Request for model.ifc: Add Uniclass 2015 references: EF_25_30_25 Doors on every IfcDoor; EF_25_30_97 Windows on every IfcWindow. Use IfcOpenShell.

First a look at what the model holds.

```python
import ifcopenshell

model = ifcopenshell.open("model.ifc")
print(model.schema)
print("classifications:", [c.Name for c in model.by_type("IfcClassification")])
for ifc_class in ("IfcDoor", "IfcRoof", "IfcStair", "IfcWall", "IfcWindow"):
    print(ifc_class, len(model.by_type(ifc_class)))
```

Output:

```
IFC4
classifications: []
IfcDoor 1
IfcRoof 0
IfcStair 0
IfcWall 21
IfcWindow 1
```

```python
import ifcopenshell
import ifcopenshell.api.classification

model = ifcopenshell.open("model.ifc")

system = ifcopenshell.api.classification.add_classification(model, classification="Uniclass 2015")

codes = {
    "IfcDoor": ("EF_25_30_25", "Doors"),
    "IfcWindow": ("EF_25_30_97", "Windows"),
}
for ifc_class, (code, name) in codes.items():
    products = model.by_type(ifc_class)
    ifcopenshell.api.classification.add_reference(
        model, products=products, classification=system, identification=code, name=name
    )
    print(code, len(products))

model.write("model-out.ifc")
```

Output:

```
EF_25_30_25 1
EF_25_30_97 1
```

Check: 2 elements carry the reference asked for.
